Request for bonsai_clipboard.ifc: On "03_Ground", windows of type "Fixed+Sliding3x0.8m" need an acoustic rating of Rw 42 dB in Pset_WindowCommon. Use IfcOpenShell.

First a look at what the model holds.

```python
import ifcopenshell
import ifcopenshell.util.element

model = ifcopenshell.open("bonsai_clipboard.ifc")
print(model.schema)
storey = next(s for s in model.by_type("IfcBuildingStorey") if s.Name == "03_Ground")
windows = [e for e in ifcopenshell.util.element.get_decomposition(storey) if e.is_a("IfcWindow")]
seen = {}
for e in windows:
    element_type = ifcopenshell.util.element.get_type(e)
    key = (element_type.Name if element_type != e and element_type else None, ifcopenshell.util.element.get_pset(e, "Pset_WindowCommon", "AcousticRating"))
    seen[key] = seen.get(key, 0) + 1
for (name, value), count in sorted(seen.items(), key=str):
    print(count, "x", name, "|", value)
```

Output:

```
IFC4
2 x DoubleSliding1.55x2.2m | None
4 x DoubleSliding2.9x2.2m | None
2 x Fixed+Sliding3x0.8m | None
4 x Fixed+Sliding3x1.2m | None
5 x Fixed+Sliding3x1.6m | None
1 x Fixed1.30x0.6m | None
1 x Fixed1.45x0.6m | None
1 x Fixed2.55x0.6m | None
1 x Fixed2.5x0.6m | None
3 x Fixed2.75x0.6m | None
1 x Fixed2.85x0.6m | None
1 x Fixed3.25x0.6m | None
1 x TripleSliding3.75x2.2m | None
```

```python
import ifcopenshell
import ifcopenshell.api.pset
import ifcopenshell.util.element

model = ifcopenshell.open("bonsai_clipboard.ifc")

storey = next(s for s in model.by_type("IfcBuildingStorey") if s.Name == "03_Ground")
windows = [e for e in ifcopenshell.util.element.get_decomposition(storey) if e.is_a("IfcWindow")]

count = 0
for e in windows:
    element_type = ifcopenshell.util.element.get_type(e)
    if element_type in (None, e) or element_type.Name != "Fixed+Sliding3x0.8m":
        continue
    # add_pset returns the element's existing set when there is one.
    pset = ifcopenshell.api.pset.add_pset(model, product=e, name="Pset_WindowCommon")
    ifcopenshell.api.pset.edit_pset(model, pset=pset, properties={"AcousticRating": "Rw 42 dB"})
    count += 1

print(count, "windows updated")

model.write("bonsai_clipboard_rev.ifc")
```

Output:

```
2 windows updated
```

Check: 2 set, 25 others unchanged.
